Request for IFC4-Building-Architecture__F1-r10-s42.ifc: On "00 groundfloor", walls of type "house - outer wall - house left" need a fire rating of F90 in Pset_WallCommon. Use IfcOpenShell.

First a look at what the model holds.

```python
import ifcopenshell
import ifcopenshell.util.element

model = ifcopenshell.open("IFC4-Building-Architecture__F1-r10-s42.ifc")
print(model.schema)
storey = next(s for s in model.by_type("IfcBuildingStorey") if s.Name == "00 groundfloor")
walls = [e for e in ifcopenshell.util.element.get_decomposition(storey) if e.is_a("IfcWall")]
seen = {}
for e in walls:
    element_type = ifcopenshell.util.element.get_type(e)
    key = (element_type.Name if element_type != e and element_type else None, ifcopenshell.util.element.get_pset(e, "Pset_WallCommon", "FireRating"))
    seen[key] = seen.get(key, 0) + 1
for (name, value), count in sorted(seen.items(), key=str):
    print(count, "x", name, "|", value)
```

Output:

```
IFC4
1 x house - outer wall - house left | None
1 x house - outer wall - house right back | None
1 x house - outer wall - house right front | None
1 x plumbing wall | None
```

```python
import ifcopenshell
import ifcopenshell.api.pset
import ifcopenshell.util.element

model = ifcopenshell.open("IFC4-Building-Architecture__F1-r10-s42.ifc")

storey = next(s for s in model.by_type("IfcBuildingStorey") if s.Name == "00 groundfloor")
walls = [e for e in ifcopenshell.util.element.get_decomposition(storey) if e.is_a("IfcWall")]

count = 0
for e in walls:
    element_type = ifcopenshell.util.element.get_type(e)
    if element_type in (None, e) or element_type.Name != "house - outer wall - house left":
        continue
    # add_pset returns the element's existing set when there is one.
    pset = ifcopenshell.api.pset.add_pset(model, product=e, name="Pset_WallCommon")
    ifcopenshell.api.pset.edit_pset(model, pset=pset, properties={"FireRating": "F90"})
    count += 1

print(count, "walls updated")

model.write("IFC4-Building-Architecture__F1-r10-s42_rev.ifc")
```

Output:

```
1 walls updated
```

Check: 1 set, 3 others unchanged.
